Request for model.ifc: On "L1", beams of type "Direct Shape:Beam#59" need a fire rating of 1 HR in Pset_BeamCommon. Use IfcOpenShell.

First a look at what the model holds.

```python
import ifcopenshell
import ifcopenshell.util.element

model = ifcopenshell.open("model.ifc")
print(model.schema)
storey = next(s for s in model.by_type("IfcBuildingStorey") if s.Name == "L1")
beams = [e for e in ifcopenshell.util.element.get_decomposition(storey) if e.is_a("IfcBeam")]
seen = {}
for e in beams:
    element_type = ifcopenshell.util.element.get_type(e)
    key = (element_type.Name if element_type != e and element_type else None, ifcopenshell.util.element.get_pset(e, "Pset_BeamCommon", "FireRating"))
    seen[key] = seen.get(key, 0) + 1
for (name, value), count in sorted(seen.items(), key=str):
    print(count, "x", name, "|", value)
```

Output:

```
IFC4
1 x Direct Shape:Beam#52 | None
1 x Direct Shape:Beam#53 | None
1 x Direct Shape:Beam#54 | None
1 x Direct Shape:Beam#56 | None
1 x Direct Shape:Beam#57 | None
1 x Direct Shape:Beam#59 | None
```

```python
import ifcopenshell
import ifcopenshell.api.pset
import ifcopenshell.util.element

model = ifcopenshell.open("model.ifc")

storey = next(s for s in model.by_type("IfcBuildingStorey") if s.Name == "L1")
beams = [e for e in ifcopenshell.util.element.get_decomposition(storey) if e.is_a("IfcBeam")]

count = 0
for e in beams:
    element_type = ifcopenshell.util.element.get_type(e)
    if element_type in (None, e) or element_type.Name != "Direct Shape:Beam#59":
        continue
    # add_pset returns the element's existing set when there is one.
    pset = ifcopenshell.api.pset.add_pset(model, product=e, name="Pset_BeamCommon")
    ifcopenshell.api.pset.edit_pset(model, pset=pset, properties={"FireRating": "1 HR"})
    count += 1

print(count, "beams updated")

model.write("model_rev.ifc")
```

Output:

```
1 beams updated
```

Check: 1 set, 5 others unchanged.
